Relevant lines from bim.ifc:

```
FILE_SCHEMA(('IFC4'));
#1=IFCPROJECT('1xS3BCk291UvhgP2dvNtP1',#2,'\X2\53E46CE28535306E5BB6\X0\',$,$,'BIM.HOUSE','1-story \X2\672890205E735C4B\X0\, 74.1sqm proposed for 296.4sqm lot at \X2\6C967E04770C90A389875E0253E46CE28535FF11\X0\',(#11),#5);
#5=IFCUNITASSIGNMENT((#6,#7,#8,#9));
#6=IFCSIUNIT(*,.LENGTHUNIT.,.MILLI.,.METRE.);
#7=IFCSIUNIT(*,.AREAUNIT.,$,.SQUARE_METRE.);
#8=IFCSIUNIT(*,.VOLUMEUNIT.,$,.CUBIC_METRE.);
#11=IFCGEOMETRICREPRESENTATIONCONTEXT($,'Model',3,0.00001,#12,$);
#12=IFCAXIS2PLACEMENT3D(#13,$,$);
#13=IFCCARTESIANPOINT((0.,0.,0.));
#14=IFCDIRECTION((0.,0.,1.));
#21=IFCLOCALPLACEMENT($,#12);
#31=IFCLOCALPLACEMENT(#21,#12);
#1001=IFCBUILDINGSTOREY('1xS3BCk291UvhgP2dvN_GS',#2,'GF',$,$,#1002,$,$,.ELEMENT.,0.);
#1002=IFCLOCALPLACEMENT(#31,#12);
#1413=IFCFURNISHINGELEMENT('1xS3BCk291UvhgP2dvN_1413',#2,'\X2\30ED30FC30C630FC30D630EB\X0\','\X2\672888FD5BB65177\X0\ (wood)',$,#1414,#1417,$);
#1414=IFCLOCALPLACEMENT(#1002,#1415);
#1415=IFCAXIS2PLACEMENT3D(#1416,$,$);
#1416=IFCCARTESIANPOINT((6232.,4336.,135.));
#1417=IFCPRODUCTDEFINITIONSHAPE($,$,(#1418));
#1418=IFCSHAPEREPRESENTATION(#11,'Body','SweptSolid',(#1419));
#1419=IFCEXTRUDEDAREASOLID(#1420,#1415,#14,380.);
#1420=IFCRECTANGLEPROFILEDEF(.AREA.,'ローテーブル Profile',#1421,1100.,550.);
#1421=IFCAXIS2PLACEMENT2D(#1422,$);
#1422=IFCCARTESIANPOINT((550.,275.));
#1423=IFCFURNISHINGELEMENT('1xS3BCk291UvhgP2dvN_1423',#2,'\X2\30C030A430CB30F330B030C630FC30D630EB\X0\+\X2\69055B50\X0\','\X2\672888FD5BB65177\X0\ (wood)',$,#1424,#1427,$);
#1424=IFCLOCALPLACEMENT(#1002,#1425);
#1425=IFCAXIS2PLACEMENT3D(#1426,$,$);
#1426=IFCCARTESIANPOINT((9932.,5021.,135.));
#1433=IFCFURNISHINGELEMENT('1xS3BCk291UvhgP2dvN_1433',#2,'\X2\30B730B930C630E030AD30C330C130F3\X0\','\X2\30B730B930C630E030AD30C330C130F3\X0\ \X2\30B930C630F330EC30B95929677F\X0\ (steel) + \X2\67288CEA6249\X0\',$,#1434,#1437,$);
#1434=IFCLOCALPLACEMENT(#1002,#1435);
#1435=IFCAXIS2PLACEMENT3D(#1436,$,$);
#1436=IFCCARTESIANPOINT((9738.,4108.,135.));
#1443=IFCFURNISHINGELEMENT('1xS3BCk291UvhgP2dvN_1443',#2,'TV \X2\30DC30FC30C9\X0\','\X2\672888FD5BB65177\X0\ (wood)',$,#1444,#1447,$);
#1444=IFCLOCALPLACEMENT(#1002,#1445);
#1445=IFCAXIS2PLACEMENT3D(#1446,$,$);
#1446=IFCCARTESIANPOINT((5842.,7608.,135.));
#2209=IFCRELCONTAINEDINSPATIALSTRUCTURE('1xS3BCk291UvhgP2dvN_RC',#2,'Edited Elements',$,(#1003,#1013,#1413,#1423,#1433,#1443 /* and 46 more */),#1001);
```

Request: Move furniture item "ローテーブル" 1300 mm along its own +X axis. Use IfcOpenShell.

```python
import ifcopenshell
import ifcopenshell.api.geometry
import ifcopenshell.util.placement
import ifcopenshell.util.unit

model = ifcopenshell.open("bim.ifc")
unit_scale = ifcopenshell.util.unit.calculate_unit_scale(model)

item = model.by_guid("1xS3BCk291UvhgP2dvN_1413")
matrix = ifcopenshell.util.placement.get_local_placement(item.ObjectPlacement)
matrix[:3, 3] += matrix[:3, 0] * 1.3 / unit_scale
ifcopenshell.api.geometry.edit_object_placement(model, product=item, matrix=matrix, is_si=False)

print(ifcopenshell.util.placement.get_local_placement(item.ObjectPlacement).round(3) + 0.0)

model.write("bim_v2.ifc")
```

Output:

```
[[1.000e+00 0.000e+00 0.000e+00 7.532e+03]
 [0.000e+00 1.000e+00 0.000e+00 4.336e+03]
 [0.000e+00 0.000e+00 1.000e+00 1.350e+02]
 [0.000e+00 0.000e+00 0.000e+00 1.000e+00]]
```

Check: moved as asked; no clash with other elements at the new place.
